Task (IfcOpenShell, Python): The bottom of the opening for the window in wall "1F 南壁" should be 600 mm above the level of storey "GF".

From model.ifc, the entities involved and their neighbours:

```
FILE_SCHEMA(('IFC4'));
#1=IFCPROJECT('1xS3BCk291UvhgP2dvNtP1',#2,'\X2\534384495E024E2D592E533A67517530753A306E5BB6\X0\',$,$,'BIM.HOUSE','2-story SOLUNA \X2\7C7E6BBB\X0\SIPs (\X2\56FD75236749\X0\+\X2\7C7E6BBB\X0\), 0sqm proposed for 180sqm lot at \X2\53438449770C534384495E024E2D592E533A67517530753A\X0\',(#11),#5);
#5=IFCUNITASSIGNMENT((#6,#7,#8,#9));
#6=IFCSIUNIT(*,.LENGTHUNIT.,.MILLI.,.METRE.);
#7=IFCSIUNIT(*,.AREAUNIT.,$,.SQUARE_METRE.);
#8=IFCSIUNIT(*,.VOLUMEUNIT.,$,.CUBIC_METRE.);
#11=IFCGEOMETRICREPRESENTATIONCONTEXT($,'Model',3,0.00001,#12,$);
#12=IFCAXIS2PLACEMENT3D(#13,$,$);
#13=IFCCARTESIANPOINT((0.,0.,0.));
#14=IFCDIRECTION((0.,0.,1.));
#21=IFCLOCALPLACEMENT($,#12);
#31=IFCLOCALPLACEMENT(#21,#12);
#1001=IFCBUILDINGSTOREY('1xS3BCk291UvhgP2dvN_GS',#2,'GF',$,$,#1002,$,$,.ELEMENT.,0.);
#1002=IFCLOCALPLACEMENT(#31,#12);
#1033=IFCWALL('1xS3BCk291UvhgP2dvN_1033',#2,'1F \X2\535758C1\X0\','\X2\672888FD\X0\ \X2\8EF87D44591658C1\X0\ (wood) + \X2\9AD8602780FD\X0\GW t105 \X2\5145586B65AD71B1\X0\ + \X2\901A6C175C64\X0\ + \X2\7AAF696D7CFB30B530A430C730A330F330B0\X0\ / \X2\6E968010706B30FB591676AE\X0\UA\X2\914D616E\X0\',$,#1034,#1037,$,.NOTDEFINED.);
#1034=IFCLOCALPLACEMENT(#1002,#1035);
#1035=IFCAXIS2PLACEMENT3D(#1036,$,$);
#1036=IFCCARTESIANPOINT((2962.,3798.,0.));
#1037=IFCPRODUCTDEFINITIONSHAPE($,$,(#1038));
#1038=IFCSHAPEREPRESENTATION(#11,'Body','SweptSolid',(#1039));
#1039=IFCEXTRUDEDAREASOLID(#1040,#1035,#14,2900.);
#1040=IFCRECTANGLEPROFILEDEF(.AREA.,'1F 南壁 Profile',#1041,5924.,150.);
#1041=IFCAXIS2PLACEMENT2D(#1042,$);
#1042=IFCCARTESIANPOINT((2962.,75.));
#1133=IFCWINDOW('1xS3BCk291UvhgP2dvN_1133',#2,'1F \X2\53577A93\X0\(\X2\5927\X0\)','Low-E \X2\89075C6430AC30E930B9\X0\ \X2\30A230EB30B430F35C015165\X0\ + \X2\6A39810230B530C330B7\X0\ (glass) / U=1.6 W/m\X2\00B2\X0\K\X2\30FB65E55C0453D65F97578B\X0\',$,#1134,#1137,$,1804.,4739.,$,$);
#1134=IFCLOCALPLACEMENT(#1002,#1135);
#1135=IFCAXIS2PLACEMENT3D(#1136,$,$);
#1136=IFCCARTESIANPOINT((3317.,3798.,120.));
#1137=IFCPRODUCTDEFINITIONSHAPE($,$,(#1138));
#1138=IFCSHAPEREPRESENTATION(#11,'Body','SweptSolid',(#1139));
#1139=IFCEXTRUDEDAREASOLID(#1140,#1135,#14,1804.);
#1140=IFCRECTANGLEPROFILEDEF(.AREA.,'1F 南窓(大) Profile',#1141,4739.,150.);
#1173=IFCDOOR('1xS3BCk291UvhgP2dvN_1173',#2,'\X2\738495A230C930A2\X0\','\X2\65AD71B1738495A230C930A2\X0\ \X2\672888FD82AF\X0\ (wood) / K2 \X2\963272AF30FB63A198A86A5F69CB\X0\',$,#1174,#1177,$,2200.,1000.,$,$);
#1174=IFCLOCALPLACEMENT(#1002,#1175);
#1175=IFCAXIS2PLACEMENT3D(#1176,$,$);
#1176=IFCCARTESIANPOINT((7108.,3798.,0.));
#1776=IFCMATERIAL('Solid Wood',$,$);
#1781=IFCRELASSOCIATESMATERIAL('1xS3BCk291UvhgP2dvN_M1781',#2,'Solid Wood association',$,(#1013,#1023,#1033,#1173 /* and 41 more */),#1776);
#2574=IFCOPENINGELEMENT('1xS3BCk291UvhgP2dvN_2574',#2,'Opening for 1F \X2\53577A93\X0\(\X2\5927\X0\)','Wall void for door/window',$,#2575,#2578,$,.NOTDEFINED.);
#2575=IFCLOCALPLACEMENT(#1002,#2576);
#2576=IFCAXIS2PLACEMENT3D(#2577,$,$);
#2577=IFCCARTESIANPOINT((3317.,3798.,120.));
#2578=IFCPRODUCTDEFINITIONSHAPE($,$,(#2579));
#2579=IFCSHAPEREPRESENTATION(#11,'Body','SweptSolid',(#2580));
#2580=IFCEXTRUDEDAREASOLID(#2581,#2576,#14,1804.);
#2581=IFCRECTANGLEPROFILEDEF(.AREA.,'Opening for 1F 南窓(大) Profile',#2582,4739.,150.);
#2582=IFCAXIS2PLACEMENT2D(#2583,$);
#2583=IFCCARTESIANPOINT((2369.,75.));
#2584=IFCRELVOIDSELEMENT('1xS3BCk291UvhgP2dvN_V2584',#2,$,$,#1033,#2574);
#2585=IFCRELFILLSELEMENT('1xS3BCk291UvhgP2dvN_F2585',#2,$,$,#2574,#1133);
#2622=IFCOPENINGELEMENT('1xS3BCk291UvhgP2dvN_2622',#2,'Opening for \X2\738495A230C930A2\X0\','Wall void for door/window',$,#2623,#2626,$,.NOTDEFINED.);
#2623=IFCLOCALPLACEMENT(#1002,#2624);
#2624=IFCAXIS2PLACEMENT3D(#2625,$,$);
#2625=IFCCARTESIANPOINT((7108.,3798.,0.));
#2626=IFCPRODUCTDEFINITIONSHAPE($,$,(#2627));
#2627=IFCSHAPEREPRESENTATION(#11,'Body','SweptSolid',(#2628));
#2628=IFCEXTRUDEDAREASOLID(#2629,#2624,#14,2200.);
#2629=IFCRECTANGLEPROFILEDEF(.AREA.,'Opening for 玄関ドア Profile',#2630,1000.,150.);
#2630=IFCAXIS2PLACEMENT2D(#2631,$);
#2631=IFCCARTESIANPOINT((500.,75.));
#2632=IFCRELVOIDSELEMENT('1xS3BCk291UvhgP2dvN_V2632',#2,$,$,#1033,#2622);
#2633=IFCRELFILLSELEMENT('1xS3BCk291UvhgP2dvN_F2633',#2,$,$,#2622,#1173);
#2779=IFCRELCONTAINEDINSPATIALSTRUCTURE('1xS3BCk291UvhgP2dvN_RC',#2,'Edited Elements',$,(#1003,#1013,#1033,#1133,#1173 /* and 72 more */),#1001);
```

```python
import numpy as np
import ifcopenshell
import ifcopenshell.api.geometry
import ifcopenshell.geom
import ifcopenshell.util.element
import ifcopenshell.util.placement
import ifcopenshell.util.shape
import ifcopenshell.util.unit

model = ifcopenshell.open("model.ifc")
unit_scale = ifcopenshell.util.unit.calculate_unit_scale(model)

window = model.by_guid("1xS3BCk291UvhgP2dvN_1133")
opening = window.FillsVoids[0].RelatingOpeningElement
storey = ifcopenshell.util.element.get_container(window, ifc_class="IfcBuildingStorey")
level = ifcopenshell.util.placement.get_local_placement(storey.ObjectPlacement)[2, 3]

# The opening's origin need not be at the sill, so measure its lowest point.
shape = ifcopenshell.geom.create_shape(ifcopenshell.geom.settings(), opening)
bottom = ifcopenshell.util.shape.get_shape_bottom_elevation(shape, shape.geometry) / unit_scale
dz = level + 0.6 / unit_scale - bottom

shift = np.array([0.0, 0.0, dz])
# The window is not placed relative to its opening, so move both.
for product in (opening, window):
    matrix = ifcopenshell.util.placement.get_local_placement(product.ObjectPlacement)
    matrix[:3, 3] += shift
    ifcopenshell.api.geometry.edit_object_placement(model, product=product, matrix=matrix, is_si=False)

print(f"moved by {dz * unit_scale:+.3f} m")

model.write("model_edited.ifc")
```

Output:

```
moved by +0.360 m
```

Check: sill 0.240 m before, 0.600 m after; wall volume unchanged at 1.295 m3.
